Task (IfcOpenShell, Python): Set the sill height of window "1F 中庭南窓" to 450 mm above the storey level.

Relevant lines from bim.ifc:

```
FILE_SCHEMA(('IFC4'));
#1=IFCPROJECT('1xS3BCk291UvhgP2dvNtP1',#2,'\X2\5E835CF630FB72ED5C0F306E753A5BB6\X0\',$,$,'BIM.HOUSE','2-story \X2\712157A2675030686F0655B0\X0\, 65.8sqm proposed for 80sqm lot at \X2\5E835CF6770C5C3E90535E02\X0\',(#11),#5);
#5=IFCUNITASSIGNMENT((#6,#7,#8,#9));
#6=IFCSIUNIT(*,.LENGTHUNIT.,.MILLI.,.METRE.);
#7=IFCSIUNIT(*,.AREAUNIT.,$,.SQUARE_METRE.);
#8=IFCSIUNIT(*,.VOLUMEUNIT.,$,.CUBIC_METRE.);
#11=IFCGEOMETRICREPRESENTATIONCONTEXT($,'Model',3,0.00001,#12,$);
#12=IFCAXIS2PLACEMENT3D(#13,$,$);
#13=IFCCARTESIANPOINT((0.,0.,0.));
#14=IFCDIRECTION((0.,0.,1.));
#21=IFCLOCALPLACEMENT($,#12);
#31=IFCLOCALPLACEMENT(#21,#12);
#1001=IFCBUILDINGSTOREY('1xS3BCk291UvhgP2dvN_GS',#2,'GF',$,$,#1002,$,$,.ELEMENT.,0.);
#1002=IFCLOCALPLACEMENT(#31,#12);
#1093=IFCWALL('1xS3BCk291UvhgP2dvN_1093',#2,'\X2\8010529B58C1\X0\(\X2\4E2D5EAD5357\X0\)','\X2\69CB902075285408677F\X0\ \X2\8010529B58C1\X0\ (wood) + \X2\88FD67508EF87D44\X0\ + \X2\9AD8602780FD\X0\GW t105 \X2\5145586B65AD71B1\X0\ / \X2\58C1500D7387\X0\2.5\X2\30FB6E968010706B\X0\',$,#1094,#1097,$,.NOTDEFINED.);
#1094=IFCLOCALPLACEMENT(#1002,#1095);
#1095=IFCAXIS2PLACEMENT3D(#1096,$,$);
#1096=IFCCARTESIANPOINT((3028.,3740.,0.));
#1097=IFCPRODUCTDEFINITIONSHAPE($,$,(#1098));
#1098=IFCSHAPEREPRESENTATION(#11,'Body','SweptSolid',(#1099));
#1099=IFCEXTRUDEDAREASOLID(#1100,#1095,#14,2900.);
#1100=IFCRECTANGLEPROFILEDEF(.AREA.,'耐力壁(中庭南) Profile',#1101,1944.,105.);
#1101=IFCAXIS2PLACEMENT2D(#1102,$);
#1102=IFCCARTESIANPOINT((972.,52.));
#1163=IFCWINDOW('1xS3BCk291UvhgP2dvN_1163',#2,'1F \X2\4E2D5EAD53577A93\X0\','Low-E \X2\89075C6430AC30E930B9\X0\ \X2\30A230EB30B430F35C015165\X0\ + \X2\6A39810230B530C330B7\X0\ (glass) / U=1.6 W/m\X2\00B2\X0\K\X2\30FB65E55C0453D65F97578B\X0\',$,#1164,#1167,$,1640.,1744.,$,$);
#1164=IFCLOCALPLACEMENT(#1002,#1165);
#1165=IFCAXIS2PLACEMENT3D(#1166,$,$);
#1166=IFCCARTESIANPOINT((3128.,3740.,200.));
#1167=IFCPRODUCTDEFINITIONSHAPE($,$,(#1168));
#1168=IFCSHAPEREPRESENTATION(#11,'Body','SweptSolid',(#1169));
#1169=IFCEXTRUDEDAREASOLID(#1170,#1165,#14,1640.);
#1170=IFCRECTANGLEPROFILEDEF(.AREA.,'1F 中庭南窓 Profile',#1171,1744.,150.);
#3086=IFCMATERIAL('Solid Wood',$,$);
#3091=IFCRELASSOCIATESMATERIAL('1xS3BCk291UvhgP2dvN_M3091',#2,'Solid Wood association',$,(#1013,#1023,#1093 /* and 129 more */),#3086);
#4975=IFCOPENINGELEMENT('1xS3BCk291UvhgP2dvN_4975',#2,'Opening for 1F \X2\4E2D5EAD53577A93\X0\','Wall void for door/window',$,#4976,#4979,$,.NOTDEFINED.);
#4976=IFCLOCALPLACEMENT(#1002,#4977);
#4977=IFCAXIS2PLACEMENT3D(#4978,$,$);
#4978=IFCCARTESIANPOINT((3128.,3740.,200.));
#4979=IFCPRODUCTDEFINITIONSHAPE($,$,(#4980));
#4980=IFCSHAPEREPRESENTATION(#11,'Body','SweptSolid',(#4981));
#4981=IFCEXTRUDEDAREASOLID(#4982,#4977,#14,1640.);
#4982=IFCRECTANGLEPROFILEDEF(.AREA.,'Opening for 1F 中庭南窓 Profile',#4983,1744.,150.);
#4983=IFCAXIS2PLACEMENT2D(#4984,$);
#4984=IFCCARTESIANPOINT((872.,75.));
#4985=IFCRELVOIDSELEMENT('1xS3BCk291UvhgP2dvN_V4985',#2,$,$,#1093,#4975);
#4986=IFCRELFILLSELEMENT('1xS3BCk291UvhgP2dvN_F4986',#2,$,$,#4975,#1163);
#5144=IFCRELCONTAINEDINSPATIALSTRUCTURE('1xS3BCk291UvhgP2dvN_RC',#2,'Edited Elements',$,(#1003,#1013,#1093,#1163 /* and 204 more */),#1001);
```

```python
import numpy as np
import ifcopenshell
import ifcopenshell.api.geometry
import ifcopenshell.geom
import ifcopenshell.util.element
import ifcopenshell.util.placement
import ifcopenshell.util.shape
import ifcopenshell.util.unit

model = ifcopenshell.open("bim.ifc")
unit_scale = ifcopenshell.util.unit.calculate_unit_scale(model)

window = model.by_guid("1xS3BCk291UvhgP2dvN_1163")
opening = window.FillsVoids[0].RelatingOpeningElement
storey = ifcopenshell.util.element.get_container(window, ifc_class="IfcBuildingStorey")
level = ifcopenshell.util.placement.get_local_placement(storey.ObjectPlacement)[2, 3]

# The opening's origin need not be at the sill, so measure its lowest point.
shape = ifcopenshell.geom.create_shape(ifcopenshell.geom.settings(), opening)
bottom = ifcopenshell.util.shape.get_shape_bottom_elevation(shape, shape.geometry) / unit_scale
dz = level + 450.0 - bottom

shift = np.array([0.0, 0.0, dz])
# The window is not placed relative to its opening, so move both.
for product in (opening, window):
    matrix = ifcopenshell.util.placement.get_local_placement(product.ObjectPlacement)
    matrix[:3, 3] += shift
    ifcopenshell.api.geometry.edit_object_placement(model, product=product, matrix=matrix, is_si=False)

print(f"moved by {dz * unit_scale:+.3f} m")

model.write("bim_rev.ifc")
```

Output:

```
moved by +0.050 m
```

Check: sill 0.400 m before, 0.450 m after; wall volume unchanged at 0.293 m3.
